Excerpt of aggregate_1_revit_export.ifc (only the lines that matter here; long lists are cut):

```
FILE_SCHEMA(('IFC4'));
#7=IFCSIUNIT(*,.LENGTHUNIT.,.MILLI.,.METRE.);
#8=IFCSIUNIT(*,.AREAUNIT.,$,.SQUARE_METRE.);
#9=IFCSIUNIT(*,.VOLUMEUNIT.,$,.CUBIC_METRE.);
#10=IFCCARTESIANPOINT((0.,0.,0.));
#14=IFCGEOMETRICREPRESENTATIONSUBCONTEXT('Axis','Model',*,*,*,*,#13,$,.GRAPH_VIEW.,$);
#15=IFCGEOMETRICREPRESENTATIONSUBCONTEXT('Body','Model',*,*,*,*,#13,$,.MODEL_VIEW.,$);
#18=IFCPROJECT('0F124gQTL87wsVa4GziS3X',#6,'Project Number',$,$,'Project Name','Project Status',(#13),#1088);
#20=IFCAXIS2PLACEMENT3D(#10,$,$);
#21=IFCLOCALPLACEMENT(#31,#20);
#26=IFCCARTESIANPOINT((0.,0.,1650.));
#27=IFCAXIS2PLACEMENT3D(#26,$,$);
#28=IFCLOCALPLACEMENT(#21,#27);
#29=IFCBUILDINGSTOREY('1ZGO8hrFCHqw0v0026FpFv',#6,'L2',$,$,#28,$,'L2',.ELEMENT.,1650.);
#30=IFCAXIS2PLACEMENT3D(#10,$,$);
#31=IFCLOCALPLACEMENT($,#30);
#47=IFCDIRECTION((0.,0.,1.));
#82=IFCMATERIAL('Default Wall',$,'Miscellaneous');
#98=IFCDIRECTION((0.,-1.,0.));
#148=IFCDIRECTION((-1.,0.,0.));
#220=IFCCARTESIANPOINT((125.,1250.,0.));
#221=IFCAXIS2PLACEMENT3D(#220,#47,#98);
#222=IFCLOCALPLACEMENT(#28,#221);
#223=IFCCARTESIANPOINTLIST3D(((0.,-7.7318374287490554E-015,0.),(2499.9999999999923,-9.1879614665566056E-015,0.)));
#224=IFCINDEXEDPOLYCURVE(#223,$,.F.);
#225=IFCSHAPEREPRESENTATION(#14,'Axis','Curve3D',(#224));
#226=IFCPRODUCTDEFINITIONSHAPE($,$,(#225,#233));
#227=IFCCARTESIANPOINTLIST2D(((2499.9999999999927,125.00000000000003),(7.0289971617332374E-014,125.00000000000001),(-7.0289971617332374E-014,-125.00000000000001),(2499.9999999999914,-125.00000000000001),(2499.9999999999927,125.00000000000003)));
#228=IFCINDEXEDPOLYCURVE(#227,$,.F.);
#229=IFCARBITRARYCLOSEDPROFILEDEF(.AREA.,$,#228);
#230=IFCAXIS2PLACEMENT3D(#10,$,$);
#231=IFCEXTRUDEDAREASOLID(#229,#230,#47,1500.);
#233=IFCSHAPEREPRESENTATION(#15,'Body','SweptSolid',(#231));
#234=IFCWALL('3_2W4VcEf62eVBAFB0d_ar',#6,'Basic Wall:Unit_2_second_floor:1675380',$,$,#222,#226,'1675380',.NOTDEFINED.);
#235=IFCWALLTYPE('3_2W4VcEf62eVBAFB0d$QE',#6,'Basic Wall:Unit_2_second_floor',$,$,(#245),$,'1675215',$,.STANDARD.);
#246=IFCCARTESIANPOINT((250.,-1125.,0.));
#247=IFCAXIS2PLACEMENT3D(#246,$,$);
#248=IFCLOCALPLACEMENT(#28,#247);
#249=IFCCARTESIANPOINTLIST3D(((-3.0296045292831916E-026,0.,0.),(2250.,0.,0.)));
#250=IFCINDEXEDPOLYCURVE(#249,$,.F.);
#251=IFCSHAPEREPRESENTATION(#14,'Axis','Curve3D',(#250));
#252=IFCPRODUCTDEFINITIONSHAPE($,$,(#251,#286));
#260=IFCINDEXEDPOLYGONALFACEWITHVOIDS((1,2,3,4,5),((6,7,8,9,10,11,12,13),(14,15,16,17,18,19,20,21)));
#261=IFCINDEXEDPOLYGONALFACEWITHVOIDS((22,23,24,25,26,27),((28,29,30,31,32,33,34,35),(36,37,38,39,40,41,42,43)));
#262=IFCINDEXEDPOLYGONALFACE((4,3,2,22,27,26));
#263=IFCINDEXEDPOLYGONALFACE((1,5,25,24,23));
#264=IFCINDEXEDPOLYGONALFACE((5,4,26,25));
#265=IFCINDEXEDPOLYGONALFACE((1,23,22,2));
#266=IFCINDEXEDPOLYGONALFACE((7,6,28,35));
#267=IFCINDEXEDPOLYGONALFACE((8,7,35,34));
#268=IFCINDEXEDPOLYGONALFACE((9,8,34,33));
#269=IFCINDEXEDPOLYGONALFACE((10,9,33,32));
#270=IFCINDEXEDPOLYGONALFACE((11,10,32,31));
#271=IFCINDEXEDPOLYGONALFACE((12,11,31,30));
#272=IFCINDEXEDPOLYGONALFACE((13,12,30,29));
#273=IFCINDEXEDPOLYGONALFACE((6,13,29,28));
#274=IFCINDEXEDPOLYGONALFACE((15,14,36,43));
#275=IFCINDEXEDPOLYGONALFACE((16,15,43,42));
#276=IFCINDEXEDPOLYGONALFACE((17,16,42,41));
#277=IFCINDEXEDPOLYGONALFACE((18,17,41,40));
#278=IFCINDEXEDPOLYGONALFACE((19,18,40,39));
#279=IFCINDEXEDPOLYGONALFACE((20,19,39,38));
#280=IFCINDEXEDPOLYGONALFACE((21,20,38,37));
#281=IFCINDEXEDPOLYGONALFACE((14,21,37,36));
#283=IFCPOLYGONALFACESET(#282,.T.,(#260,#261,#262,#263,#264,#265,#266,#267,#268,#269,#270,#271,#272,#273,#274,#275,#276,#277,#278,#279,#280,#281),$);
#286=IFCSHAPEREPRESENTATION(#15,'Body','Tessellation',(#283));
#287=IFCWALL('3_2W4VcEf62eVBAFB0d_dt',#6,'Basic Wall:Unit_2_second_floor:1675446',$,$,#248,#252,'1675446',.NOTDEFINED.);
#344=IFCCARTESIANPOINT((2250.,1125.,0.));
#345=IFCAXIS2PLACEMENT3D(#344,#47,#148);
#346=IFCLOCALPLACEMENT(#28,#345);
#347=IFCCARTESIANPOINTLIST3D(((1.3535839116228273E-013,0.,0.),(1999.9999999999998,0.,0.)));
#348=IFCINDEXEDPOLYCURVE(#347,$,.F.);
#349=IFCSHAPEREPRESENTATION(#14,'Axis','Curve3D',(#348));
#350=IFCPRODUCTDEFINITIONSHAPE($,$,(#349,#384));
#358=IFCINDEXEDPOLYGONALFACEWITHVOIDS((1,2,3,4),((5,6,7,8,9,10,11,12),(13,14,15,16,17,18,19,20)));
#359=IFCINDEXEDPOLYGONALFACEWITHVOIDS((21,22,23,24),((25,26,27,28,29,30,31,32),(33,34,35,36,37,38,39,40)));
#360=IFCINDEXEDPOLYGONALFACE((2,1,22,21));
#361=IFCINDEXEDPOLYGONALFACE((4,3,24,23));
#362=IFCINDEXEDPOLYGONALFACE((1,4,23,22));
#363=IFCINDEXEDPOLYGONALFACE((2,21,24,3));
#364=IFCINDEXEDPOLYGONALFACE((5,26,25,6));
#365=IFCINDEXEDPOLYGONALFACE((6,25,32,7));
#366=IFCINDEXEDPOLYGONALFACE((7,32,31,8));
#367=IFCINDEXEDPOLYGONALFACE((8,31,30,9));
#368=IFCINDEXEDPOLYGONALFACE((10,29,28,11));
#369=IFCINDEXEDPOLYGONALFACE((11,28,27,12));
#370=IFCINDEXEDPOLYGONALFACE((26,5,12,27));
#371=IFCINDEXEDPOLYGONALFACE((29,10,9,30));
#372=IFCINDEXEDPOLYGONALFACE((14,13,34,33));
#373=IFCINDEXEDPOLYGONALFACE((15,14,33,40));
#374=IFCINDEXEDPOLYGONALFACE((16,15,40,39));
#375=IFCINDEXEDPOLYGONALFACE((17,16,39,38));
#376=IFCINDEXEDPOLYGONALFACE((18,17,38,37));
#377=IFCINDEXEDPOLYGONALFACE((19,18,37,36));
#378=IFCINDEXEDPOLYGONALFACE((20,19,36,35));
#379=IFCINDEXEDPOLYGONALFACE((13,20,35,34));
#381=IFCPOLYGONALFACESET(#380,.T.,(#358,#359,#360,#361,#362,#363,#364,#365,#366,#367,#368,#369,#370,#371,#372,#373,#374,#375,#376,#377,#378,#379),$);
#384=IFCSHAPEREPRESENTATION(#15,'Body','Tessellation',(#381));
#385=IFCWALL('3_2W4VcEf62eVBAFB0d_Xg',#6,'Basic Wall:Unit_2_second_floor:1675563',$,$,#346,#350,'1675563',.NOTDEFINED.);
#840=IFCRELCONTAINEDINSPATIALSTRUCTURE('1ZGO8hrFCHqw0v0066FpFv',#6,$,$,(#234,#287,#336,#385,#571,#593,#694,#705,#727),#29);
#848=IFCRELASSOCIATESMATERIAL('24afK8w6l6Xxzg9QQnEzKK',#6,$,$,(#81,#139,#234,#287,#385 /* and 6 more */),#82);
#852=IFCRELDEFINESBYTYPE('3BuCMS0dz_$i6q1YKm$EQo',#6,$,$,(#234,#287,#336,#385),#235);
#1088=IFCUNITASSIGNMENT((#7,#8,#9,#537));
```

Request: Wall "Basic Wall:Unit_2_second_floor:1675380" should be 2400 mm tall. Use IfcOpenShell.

```python
import ifcopenshell
import ifcopenshell.geom
import ifcopenshell.util.representation
import ifcopenshell.util.shape
import ifcopenshell.util.unit

model = ifcopenshell.open("aggregate_1_revit_export.ifc")
unit_scale = ifcopenshell.util.unit.calculate_unit_scale(model)
settings = ifcopenshell.geom.settings()


def volume(element):
    """Net volume in cubic metres, openings subtracted."""
    shape = ifcopenshell.geom.create_shape(settings, element)
    return ifcopenshell.util.shape.get_volume(shape.geometry)


wall = model.by_id(234)
before = volume(wall)

body = ifcopenshell.util.representation.get_representation(wall, "Model", "Body")
solid = body.Items[0]
old_height = solid.Depth
solid.Depth = 2.4 / unit_scale
after = volume(wall)

print(f"height {old_height:g} -> {solid.Depth:g}, volume {before:.3f} -> {after:.3f} m3")

model.write("aggregate_1_revit_export-out.ifc")
```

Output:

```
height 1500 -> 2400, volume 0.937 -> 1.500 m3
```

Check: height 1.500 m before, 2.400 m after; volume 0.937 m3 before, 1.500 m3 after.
